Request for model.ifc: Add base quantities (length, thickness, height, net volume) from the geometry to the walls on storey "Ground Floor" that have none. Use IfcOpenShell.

First a look at what the model holds.

```python
import ifcopenshell
import ifcopenshell.util.element
import ifcopenshell.util.unit

model = ifcopenshell.open("model.ifc")
print(model.schema)
for unit_type in ("LENGTHUNIT", "AREAUNIT", "VOLUMEUNIT"):
    print(unit_type, ifcopenshell.util.unit.calculate_unit_scale(model, unit_type))
storey = next(s for s in model.by_type("IfcBuildingStorey") if s.Name == "Ground Floor")
walls = [e for e in ifcopenshell.util.element.get_decomposition(storey) if e.is_a("IfcWall")]
for e in sorted(walls, key=lambda e: e.id()):
    print(e.id(), e.is_a(), e.Name, list(ifcopenshell.util.element.get_psets(e, qtos_only=True)), sep=" | ")
```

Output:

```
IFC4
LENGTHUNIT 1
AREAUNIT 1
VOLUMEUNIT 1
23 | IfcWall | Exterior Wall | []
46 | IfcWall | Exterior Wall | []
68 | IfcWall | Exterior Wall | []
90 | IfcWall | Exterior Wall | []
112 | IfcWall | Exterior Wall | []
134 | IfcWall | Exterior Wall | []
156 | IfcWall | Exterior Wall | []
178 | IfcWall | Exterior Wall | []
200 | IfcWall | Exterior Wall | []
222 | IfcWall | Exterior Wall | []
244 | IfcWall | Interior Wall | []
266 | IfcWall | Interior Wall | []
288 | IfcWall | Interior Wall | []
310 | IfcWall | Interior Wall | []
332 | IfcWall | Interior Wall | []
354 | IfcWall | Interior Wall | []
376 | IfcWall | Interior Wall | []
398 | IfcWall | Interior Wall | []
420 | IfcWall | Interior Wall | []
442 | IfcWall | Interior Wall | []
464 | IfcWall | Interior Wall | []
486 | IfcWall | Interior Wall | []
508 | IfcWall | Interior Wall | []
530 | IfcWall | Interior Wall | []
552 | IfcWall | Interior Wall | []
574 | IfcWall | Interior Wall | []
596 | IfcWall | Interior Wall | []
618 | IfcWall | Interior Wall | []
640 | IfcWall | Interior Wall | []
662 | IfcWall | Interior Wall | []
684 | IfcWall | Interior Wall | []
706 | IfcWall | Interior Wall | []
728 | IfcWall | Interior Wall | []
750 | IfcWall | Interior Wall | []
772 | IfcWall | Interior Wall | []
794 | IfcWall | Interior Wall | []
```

```python
import ifcopenshell
import ifcopenshell.api.pset
import ifcopenshell.geom
import ifcopenshell.util.element
import ifcopenshell.util.shape
import ifcopenshell.util.unit

model = ifcopenshell.open("model.ifc")
unit_scale = ifcopenshell.util.unit.calculate_unit_scale(model)
volume_scale = ifcopenshell.util.unit.calculate_unit_scale(model, "VOLUMEUNIT")
settings = ifcopenshell.geom.settings()

storey = next(s for s in model.by_type("IfcBuildingStorey") if s.Name == "Ground Floor")
walls = [e for e in ifcopenshell.util.element.get_decomposition(storey) if e.is_a("IfcWall")]

for e in sorted(walls, key=lambda e: e.id()):
    if ifcopenshell.util.element.get_psets(e, qtos_only=True, should_inherit=False):
        continue
    # Geometry comes back in metres, in the element's own axes.
    shape = ifcopenshell.geom.create_shape(settings, e)
    values = {
        "Length": ifcopenshell.util.shape.get_x(shape.geometry) / unit_scale,
        "Width": ifcopenshell.util.shape.get_y(shape.geometry) / unit_scale,
        "Height": ifcopenshell.util.shape.get_z(shape.geometry) / unit_scale,
        "NetVolume": ifcopenshell.util.shape.get_volume(shape.geometry) / volume_scale,
    }
    qto = ifcopenshell.api.pset.add_qto(model, product=e, name="Qto_WallBaseQuantities")
    ifcopenshell.api.pset.edit_qto(model, qto=qto, properties=values)
    print(e.id(), {k: round(v, 3) for k, v in values.items()})

model.write("model_v2.ifc")
```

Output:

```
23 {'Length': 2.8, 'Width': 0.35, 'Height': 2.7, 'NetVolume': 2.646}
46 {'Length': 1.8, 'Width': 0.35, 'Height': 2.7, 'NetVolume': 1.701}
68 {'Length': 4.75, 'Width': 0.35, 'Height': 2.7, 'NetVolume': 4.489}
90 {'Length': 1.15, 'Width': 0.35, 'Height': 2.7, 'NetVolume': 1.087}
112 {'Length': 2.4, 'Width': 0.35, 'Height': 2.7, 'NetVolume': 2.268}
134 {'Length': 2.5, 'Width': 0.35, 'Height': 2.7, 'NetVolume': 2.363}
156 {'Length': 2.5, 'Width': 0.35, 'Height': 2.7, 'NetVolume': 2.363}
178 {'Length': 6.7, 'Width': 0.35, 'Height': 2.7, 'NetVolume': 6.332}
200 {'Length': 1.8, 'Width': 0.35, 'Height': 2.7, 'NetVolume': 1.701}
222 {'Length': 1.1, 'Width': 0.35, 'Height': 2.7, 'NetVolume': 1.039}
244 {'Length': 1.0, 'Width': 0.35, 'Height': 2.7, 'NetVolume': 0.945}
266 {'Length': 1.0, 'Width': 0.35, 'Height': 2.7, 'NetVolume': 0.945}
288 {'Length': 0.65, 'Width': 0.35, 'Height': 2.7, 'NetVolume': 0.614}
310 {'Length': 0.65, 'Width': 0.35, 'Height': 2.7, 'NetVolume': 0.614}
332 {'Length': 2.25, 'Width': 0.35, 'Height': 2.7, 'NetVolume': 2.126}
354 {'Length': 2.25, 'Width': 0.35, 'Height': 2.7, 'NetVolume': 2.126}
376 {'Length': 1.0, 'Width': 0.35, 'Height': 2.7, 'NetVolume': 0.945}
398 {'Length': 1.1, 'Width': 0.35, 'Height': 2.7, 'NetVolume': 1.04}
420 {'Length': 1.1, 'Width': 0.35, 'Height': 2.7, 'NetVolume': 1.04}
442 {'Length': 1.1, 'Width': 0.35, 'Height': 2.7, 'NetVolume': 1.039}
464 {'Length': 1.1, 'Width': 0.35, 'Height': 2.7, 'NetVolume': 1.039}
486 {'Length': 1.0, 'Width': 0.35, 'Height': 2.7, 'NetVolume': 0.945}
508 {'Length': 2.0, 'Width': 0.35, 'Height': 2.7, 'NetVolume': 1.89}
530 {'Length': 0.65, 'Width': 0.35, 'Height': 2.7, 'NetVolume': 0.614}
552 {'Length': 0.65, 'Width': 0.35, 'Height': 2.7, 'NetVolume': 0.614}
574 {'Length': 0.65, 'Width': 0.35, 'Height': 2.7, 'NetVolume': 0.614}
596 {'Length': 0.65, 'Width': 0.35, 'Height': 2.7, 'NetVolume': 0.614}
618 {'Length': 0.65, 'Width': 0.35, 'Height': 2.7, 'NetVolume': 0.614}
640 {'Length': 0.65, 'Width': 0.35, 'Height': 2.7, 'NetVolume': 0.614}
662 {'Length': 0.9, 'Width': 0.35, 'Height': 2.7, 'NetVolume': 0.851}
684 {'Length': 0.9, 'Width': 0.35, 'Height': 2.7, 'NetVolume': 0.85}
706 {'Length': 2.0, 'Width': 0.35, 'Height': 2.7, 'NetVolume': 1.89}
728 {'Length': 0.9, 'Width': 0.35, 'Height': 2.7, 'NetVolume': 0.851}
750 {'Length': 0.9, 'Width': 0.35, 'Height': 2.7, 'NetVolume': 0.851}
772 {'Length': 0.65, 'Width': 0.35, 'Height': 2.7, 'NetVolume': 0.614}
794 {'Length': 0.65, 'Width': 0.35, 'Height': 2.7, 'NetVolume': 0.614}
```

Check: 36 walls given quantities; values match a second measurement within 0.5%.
